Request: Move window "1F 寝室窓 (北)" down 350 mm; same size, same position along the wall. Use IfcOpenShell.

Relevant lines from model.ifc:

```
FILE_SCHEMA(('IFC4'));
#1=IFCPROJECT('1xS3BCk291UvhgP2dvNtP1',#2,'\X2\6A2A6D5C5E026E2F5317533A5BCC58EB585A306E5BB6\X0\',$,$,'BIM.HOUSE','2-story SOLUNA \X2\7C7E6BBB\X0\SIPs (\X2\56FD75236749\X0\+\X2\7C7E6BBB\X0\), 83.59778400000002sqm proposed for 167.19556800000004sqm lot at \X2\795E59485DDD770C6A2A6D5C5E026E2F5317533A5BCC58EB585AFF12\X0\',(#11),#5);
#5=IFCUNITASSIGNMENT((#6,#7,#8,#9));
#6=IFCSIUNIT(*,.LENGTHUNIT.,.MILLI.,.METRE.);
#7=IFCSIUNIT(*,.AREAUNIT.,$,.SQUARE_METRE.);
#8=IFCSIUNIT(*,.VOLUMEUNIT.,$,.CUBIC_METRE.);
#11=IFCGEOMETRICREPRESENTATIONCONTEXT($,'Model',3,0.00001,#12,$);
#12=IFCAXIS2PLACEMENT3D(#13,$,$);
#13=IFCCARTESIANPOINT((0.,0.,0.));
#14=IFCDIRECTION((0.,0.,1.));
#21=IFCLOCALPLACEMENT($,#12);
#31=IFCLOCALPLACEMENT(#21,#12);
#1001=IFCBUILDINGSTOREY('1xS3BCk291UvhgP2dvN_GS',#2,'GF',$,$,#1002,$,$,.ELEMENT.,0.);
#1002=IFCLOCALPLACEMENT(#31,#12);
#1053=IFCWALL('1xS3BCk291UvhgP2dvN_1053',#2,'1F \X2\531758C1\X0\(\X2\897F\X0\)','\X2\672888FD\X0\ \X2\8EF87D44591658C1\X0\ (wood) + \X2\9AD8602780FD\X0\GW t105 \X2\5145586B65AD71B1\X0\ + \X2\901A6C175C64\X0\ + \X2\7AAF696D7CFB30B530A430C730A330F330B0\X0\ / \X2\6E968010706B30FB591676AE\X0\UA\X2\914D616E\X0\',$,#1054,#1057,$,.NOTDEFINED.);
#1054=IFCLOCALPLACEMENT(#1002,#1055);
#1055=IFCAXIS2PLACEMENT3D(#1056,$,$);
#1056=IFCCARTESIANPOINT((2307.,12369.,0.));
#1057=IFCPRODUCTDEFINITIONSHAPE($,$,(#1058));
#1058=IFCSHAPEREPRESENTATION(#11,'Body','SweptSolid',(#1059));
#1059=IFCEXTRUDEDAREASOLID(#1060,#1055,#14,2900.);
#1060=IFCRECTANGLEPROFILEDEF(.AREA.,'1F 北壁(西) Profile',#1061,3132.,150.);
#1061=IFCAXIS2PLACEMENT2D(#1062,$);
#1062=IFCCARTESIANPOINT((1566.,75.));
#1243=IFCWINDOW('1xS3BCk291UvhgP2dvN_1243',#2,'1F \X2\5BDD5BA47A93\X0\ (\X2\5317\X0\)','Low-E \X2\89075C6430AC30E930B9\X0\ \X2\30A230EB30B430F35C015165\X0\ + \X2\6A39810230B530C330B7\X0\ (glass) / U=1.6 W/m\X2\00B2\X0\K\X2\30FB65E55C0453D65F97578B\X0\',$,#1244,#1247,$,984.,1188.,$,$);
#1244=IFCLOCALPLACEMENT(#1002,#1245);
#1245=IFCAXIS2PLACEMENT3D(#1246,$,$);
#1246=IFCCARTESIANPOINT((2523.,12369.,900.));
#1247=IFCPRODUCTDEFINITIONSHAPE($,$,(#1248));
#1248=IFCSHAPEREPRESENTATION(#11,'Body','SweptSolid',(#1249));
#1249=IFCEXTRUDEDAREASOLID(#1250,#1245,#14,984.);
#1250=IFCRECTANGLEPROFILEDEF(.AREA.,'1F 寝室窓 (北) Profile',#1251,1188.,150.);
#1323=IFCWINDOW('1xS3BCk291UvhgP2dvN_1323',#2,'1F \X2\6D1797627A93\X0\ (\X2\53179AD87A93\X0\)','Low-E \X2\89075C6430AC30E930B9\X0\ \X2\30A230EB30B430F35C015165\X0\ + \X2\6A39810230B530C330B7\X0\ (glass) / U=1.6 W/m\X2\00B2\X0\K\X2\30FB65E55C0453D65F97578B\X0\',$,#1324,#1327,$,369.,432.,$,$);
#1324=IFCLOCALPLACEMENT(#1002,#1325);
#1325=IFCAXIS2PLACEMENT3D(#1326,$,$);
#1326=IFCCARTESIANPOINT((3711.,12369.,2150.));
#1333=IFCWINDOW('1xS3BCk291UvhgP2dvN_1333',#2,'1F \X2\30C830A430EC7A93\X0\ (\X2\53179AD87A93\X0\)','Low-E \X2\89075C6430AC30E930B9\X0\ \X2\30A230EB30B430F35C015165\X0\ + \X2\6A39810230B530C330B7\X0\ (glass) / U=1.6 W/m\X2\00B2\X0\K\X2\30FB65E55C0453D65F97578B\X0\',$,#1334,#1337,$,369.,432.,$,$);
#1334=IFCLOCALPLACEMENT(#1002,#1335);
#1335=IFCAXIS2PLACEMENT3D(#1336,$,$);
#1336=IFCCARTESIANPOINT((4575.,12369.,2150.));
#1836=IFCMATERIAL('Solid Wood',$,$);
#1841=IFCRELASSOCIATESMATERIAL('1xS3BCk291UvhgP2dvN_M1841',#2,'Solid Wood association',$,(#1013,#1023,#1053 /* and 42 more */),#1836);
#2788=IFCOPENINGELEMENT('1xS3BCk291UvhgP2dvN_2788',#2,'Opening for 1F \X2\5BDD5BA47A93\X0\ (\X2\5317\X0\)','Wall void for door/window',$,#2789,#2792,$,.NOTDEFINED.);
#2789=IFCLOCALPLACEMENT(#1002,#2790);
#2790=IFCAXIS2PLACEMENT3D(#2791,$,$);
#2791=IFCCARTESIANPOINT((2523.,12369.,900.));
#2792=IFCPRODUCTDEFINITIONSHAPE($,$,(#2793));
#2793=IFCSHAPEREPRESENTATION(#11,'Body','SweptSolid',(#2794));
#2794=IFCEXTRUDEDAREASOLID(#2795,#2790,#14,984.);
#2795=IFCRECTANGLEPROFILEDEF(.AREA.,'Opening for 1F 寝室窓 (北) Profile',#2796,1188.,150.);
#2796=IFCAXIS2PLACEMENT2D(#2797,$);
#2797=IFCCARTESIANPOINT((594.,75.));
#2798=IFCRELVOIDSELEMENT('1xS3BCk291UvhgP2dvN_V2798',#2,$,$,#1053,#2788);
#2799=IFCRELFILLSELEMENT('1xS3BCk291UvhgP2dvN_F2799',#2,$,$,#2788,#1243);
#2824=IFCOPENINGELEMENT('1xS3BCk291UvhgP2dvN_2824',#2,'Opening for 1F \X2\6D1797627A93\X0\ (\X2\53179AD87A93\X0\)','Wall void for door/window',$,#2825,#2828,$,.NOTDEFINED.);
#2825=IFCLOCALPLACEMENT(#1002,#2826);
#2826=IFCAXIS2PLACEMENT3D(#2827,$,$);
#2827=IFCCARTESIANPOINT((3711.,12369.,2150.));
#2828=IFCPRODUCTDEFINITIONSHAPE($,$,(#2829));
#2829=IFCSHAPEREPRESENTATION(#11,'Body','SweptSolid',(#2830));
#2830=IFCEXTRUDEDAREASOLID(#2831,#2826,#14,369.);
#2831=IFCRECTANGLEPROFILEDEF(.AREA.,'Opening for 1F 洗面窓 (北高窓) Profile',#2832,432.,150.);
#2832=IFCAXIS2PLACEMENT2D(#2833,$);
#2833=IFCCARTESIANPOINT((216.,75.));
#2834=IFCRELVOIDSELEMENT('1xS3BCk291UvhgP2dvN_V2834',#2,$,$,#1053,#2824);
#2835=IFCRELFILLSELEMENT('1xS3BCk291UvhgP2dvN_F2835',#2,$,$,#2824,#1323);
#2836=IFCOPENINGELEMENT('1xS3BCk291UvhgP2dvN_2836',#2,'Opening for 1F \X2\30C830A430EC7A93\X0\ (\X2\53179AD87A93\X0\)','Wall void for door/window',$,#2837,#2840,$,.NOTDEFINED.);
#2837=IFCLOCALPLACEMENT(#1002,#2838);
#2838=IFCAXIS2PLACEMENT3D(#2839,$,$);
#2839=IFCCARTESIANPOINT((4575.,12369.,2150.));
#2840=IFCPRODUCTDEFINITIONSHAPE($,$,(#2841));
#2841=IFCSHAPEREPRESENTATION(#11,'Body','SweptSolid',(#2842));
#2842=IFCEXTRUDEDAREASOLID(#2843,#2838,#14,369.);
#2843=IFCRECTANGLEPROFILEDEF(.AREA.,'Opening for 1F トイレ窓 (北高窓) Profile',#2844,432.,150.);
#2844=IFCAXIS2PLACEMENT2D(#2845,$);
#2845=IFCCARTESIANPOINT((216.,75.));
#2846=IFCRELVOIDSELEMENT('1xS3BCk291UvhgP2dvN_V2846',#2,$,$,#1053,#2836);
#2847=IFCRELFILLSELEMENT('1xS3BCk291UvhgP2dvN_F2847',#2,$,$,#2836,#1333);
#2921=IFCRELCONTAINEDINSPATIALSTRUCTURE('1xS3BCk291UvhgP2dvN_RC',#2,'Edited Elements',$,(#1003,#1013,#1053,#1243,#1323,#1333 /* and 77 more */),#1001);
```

```python
import numpy as np
import ifcopenshell
import ifcopenshell.api.geometry
import ifcopenshell.util.placement
import ifcopenshell.util.unit

model = ifcopenshell.open("model.ifc")
unit_scale = ifcopenshell.util.unit.calculate_unit_scale(model)

window = model.by_id(1243)
opening = window.FillsVoids[0].RelatingOpeningElement
dz = -0.35 / unit_scale

shift = np.array([0.0, 0.0, dz])
# The window is not placed relative to its opening, so move both.
for product in (opening, window):
    matrix = ifcopenshell.util.placement.get_local_placement(product.ObjectPlacement)
    matrix[:3, 3] += shift
    ifcopenshell.api.geometry.edit_object_placement(model, product=product, matrix=matrix, is_si=False)

print(f"moved by {dz * unit_scale:+.3f} m")

model.write("model_updated.ifc")
```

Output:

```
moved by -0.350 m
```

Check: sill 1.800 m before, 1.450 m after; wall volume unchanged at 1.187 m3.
